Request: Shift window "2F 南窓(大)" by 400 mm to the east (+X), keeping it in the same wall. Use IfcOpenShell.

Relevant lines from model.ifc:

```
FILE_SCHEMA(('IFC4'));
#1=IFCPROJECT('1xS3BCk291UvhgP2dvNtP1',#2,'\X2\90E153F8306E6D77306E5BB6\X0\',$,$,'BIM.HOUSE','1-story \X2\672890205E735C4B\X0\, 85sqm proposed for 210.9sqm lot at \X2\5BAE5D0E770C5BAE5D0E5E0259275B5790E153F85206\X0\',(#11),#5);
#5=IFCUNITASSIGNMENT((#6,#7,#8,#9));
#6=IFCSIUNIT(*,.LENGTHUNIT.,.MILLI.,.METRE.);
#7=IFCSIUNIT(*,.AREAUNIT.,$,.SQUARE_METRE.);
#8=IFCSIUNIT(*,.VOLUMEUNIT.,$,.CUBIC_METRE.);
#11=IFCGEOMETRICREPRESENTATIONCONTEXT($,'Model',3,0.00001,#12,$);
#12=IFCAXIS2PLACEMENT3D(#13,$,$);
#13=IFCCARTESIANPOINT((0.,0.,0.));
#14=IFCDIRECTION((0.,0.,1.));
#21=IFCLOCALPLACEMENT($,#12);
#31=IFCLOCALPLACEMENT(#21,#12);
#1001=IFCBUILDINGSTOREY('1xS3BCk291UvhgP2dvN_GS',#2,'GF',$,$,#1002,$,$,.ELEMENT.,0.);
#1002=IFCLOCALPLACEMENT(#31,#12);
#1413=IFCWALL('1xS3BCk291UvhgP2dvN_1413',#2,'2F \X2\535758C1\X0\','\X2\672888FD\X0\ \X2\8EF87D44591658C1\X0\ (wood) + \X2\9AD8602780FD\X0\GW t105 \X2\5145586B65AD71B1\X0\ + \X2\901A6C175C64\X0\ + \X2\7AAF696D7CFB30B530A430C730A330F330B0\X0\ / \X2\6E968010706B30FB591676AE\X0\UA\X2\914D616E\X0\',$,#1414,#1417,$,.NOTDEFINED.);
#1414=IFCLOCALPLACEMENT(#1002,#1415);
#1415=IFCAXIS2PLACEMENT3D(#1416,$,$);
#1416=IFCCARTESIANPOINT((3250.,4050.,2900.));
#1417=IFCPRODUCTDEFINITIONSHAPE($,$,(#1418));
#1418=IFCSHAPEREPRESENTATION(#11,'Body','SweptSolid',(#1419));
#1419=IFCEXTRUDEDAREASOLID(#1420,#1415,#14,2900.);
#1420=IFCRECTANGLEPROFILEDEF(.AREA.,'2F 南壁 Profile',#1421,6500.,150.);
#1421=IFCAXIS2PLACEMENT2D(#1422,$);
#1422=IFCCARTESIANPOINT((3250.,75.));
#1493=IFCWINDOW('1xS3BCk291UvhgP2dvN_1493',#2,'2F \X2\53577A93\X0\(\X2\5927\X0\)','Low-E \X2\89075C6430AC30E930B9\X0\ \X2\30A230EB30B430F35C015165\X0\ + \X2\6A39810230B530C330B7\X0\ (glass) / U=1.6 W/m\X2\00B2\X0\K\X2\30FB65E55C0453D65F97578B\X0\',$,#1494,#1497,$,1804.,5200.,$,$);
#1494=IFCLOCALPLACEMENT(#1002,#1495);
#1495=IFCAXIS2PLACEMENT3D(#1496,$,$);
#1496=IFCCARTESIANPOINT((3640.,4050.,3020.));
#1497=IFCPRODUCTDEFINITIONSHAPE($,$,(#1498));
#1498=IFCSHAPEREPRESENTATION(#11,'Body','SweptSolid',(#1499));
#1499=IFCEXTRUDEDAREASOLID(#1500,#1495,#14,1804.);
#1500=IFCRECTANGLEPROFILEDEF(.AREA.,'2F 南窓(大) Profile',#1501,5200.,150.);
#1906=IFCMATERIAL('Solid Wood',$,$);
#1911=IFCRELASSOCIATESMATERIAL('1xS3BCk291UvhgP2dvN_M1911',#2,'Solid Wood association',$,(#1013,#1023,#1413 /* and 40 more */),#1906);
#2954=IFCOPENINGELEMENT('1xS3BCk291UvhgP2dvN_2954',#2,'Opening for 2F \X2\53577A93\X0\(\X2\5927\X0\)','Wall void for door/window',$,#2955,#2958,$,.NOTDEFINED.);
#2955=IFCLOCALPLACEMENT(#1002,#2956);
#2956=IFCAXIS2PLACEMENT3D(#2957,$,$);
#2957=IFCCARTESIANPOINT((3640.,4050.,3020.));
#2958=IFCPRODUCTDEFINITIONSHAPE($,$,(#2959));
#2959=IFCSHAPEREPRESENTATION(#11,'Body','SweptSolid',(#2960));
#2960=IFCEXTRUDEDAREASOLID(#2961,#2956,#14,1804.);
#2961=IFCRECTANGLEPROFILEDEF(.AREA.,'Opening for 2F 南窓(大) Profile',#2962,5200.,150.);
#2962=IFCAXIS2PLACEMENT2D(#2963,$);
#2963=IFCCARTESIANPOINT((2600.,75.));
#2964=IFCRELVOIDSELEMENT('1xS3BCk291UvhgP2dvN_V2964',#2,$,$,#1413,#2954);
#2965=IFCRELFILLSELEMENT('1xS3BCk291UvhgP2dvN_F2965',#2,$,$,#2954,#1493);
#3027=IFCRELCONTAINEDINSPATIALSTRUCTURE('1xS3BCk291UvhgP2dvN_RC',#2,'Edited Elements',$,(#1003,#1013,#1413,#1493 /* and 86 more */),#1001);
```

```python
import ifcopenshell
import ifcopenshell.api.geometry
import ifcopenshell.util.placement

model = ifcopenshell.open("model.ifc")

window = model.by_guid("1xS3BCk291UvhgP2dvN_1493")
opening = window.FillsVoids[0].RelatingOpeningElement
wall = opening.VoidsElements[0].RelatingBuildingElement

wall_matrix = ifcopenshell.util.placement.get_local_placement(wall.ObjectPlacement)
shift = wall_matrix[:3, 0] * 400.0
before = ifcopenshell.util.placement.get_local_placement(window.ObjectPlacement)[:3, 3].copy()

# The window is not placed relative to its opening, so move both.
for product in (opening, window):
    matrix = ifcopenshell.util.placement.get_local_placement(product.ObjectPlacement)
    matrix[:3, 3] += shift
    ifcopenshell.api.geometry.edit_object_placement(model, product=product, matrix=matrix, is_si=False)

after = ifcopenshell.util.placement.get_local_placement(window.ObjectPlacement)[:3, 3]
print("window moved by", (after - before).round(3) + 0.0)

model.write("model_rev.ifc")
```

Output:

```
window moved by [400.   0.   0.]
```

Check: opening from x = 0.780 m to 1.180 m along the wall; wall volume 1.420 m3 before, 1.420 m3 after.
